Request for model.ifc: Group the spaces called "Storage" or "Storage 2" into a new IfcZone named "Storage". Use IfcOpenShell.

First a look at what the model holds.

```python
import ifcopenshell

model = ifcopenshell.open("model.ifc")
print(model.schema)
seen = {}
for space in model.by_type("IfcSpace"):
    seen[space.LongName] = seen.get(space.LongName, 0) + 1
for name, count in sorted(seen.items(), key=str):
    print(count, "x", name)
print("zones:", [z.Name for z in model.by_type("IfcZone")][:20])
```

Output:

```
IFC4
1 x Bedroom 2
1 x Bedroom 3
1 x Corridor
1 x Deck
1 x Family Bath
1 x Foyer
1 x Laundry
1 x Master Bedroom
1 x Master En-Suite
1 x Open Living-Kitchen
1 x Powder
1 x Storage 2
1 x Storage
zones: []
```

```python
import ifcopenshell
import ifcopenshell.api.group
import ifcopenshell.api.root

model = ifcopenshell.open("model.ifc")

names = {"Storage", "Storage 2"}
spaces = [s for s in model.by_type("IfcSpace") if s.LongName in names]

zone = ifcopenshell.api.root.create_entity(model, ifc_class="IfcZone", name="Storage")
ifcopenshell.api.group.assign_group(model, products=spaces, group=zone)
print(len(spaces), "spaces in", zone.Name)

model.write("model_v2.ifc")
```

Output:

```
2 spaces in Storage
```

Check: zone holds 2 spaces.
